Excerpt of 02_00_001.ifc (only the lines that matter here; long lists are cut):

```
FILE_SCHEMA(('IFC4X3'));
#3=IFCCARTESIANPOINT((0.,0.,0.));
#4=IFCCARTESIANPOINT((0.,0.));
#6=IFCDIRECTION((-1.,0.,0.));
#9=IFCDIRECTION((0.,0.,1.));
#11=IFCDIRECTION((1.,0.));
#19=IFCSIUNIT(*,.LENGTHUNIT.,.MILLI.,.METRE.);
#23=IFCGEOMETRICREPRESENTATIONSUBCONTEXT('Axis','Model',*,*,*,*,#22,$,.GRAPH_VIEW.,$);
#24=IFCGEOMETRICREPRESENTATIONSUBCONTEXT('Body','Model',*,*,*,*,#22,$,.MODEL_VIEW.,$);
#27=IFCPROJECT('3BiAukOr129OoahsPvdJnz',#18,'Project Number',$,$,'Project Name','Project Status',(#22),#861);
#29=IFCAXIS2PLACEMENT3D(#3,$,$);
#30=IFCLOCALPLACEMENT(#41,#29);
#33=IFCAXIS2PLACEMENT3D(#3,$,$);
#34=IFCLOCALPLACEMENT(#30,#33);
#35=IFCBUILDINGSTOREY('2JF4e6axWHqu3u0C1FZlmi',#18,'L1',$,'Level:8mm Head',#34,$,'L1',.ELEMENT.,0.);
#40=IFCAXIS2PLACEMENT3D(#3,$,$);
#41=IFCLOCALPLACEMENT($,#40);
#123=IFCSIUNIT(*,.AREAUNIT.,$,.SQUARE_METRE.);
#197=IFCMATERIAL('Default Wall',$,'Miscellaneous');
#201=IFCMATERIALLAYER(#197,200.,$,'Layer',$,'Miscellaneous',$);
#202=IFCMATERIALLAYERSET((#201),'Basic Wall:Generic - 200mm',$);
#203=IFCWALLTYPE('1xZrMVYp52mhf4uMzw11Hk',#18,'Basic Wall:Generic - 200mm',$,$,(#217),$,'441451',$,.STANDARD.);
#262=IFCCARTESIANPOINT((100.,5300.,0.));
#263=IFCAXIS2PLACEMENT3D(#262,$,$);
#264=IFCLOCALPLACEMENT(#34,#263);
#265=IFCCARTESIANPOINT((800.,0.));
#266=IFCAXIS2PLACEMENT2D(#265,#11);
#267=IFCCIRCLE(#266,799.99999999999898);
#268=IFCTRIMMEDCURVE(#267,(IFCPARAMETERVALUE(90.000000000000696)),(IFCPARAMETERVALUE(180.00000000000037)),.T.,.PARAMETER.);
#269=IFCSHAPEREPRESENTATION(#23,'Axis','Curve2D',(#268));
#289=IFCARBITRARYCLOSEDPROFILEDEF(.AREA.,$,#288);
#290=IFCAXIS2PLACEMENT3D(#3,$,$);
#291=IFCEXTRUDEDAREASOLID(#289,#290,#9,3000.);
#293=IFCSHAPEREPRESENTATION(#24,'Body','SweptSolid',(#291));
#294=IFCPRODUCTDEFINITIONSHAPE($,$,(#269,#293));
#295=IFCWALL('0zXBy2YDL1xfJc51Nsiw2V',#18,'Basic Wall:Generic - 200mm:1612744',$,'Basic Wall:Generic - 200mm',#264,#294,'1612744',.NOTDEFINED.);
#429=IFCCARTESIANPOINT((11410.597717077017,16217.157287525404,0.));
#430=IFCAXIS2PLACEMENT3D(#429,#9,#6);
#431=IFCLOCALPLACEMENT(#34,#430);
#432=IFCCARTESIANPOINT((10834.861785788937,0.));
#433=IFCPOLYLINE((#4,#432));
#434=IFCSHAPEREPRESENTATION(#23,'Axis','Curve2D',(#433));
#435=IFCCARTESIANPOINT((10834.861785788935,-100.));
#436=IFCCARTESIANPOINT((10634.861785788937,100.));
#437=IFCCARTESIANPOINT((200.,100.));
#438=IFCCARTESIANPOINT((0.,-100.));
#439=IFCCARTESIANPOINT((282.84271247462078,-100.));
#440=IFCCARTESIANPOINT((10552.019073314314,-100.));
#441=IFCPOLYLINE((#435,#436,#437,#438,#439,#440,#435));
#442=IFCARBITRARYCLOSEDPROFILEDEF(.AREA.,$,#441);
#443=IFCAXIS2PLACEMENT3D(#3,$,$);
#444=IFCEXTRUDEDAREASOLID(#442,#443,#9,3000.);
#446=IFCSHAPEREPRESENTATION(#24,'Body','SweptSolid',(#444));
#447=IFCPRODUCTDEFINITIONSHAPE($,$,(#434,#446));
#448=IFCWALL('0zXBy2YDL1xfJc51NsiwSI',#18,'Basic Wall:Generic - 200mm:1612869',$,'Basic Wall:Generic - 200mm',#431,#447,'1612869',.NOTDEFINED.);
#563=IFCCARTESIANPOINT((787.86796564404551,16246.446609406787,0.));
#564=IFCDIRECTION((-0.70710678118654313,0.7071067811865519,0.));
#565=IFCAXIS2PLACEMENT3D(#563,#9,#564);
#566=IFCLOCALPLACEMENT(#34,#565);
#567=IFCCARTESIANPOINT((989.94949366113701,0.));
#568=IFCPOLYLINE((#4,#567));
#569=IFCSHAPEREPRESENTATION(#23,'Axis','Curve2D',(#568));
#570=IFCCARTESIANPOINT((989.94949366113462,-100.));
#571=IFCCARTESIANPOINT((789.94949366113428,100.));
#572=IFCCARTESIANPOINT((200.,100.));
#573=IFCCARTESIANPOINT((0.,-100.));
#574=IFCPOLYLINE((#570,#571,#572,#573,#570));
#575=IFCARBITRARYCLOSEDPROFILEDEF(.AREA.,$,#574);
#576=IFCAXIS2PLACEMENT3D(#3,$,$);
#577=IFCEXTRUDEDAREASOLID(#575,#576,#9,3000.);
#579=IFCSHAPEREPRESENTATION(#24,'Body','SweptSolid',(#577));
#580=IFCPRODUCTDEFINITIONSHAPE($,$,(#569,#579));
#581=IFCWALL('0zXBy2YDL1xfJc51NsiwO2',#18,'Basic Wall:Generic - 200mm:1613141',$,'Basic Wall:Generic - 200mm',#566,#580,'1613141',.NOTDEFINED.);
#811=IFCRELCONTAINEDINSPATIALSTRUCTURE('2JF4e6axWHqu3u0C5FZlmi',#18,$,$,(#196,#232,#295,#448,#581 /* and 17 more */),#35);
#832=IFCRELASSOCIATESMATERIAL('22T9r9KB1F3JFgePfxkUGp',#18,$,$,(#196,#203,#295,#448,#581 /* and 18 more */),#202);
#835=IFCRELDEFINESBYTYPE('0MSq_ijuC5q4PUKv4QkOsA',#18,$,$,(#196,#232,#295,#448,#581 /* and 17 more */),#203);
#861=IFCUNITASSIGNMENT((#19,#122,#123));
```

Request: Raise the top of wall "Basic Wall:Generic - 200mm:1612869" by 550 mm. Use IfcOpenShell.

```python
import ifcopenshell
import ifcopenshell.geom
import ifcopenshell.util.representation
import ifcopenshell.util.shape
import ifcopenshell.util.unit

model = ifcopenshell.open("02_00_001.ifc")
unit_scale = ifcopenshell.util.unit.calculate_unit_scale(model)
settings = ifcopenshell.geom.settings()


def volume(element):
    """Net volume in cubic metres, openings subtracted."""
    shape = ifcopenshell.geom.create_shape(settings, element)
    return ifcopenshell.util.shape.get_volume(shape.geometry)


wall = model.by_guid("0zXBy2YDL1xfJc51NsiwSI")
before = volume(wall)

body = ifcopenshell.util.representation.get_representation(wall, "Model", "Body")
solid = body.Items[0]
old_height = solid.Depth
solid.Depth += 0.55 / unit_scale
after = volume(wall)

print(f"height {old_height:g} -> {solid.Depth:g}, volume {before:.3f} -> {after:.3f} m3")

model.write("02_00_001_updated.ifc")
```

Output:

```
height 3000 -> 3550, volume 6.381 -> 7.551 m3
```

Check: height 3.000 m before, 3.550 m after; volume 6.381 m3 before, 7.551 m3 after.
